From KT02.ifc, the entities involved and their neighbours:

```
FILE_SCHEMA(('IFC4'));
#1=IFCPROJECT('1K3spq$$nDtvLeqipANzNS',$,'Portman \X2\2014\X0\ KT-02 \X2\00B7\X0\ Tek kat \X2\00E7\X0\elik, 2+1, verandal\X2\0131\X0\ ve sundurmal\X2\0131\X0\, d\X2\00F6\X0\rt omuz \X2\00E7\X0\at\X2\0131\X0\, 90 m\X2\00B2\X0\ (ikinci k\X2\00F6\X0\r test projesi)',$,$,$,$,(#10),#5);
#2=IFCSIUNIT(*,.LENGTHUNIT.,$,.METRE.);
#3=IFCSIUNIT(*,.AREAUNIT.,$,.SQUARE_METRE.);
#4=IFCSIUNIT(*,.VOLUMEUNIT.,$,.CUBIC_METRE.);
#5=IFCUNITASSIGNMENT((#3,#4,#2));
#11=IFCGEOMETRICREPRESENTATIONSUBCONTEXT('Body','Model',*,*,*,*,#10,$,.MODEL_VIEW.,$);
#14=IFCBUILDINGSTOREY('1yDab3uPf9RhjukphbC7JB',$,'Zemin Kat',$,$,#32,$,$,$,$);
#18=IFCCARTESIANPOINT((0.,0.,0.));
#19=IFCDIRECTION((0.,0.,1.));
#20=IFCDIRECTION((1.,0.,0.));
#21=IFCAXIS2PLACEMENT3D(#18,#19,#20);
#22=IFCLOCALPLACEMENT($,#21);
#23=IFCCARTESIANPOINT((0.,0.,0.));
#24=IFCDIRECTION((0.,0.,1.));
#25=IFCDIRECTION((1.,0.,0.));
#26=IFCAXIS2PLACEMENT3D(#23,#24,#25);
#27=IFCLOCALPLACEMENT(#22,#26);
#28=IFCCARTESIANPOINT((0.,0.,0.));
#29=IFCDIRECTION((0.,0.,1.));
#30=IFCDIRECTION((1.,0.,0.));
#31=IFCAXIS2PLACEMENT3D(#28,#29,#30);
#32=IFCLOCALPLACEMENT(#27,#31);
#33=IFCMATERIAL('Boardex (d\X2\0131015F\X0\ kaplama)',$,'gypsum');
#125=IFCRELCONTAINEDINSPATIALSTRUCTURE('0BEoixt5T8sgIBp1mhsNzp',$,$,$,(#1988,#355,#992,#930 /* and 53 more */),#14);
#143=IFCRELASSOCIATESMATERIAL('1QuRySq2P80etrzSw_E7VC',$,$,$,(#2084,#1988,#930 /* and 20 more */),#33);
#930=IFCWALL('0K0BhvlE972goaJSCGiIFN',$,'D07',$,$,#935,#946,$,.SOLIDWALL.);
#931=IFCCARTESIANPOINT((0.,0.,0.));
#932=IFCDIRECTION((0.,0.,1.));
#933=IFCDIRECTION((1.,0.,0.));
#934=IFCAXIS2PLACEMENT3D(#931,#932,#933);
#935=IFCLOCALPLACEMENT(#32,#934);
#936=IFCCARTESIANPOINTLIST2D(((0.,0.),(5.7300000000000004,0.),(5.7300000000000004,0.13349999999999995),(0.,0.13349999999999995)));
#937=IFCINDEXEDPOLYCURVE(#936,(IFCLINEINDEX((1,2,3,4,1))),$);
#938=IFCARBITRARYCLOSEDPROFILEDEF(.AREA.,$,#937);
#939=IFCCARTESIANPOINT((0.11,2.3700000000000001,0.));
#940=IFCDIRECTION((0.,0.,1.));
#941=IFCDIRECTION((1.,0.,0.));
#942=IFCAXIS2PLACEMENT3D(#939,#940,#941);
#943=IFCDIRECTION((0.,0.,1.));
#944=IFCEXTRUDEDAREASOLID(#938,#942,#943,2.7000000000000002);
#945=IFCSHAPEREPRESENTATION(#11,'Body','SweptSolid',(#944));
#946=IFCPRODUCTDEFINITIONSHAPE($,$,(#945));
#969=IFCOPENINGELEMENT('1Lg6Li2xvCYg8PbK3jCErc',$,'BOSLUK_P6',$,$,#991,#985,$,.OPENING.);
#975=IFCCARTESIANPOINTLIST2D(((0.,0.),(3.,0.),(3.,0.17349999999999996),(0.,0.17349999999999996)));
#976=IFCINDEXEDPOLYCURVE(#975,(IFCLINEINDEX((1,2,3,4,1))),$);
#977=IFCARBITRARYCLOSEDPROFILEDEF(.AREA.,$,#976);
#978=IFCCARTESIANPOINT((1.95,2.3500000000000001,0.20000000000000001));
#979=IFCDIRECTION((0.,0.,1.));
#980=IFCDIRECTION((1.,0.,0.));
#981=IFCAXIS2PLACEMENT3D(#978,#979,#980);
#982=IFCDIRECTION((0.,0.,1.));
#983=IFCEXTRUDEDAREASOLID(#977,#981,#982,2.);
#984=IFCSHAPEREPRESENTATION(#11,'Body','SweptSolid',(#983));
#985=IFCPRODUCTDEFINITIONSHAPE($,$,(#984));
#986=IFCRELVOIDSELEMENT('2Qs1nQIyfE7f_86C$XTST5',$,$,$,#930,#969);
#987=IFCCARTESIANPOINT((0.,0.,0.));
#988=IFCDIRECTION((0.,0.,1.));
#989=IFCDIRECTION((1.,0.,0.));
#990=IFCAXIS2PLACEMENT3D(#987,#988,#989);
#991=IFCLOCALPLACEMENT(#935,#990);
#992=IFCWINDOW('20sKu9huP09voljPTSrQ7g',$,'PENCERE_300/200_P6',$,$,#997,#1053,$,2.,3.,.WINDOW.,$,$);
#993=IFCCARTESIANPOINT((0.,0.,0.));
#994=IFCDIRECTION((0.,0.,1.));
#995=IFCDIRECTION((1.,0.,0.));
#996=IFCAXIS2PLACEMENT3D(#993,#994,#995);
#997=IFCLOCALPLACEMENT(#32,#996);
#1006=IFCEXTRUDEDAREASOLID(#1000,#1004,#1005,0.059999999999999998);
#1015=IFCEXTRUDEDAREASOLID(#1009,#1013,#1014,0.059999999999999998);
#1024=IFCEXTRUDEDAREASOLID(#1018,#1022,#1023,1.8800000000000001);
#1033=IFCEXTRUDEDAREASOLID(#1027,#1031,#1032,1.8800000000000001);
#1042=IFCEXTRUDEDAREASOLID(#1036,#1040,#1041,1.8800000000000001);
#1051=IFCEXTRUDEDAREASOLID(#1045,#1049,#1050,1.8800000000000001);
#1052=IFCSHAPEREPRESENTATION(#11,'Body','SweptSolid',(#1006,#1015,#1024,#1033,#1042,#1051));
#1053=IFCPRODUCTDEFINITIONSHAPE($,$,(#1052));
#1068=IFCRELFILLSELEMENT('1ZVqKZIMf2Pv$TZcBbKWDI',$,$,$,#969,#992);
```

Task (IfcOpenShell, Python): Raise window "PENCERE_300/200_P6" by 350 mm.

```python
import numpy as np
import ifcopenshell
import ifcopenshell.api.geometry
import ifcopenshell.util.placement
import ifcopenshell.util.unit

model = ifcopenshell.open("KT02.ifc")
unit_scale = ifcopenshell.util.unit.calculate_unit_scale(model)

window = model.by_id(992)
opening = window.FillsVoids[0].RelatingOpeningElement
dz = 0.35 / unit_scale

shift = np.array([0.0, 0.0, dz])
# The window is not placed relative to its opening, so move both.
for product in (opening, window):
    matrix = ifcopenshell.util.placement.get_local_placement(product.ObjectPlacement)
    matrix[:3, 3] += shift
    ifcopenshell.api.geometry.edit_object_placement(model, product=product, matrix=matrix, is_si=False)

print(f"moved by {dz * unit_scale:+.3f} m")

model.write("KT02_updated.ifc")
```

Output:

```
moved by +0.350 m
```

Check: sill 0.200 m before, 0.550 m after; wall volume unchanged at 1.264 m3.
